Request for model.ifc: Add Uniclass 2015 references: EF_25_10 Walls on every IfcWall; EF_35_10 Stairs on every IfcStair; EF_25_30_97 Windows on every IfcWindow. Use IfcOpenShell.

First a look at what the model holds.

```python
import ifcopenshell

model = ifcopenshell.open("model.ifc")
print(model.schema)
print("classifications:", [c.Name for c in model.by_type("IfcClassification")])
for ifc_class in ("IfcDoor", "IfcRoof", "IfcStair", "IfcWall", "IfcWindow"):
    print(ifc_class, len(model.by_type(ifc_class)))
```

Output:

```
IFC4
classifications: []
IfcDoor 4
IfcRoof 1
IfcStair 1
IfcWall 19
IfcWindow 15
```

```python
import ifcopenshell
import ifcopenshell.api.classification

model = ifcopenshell.open("model.ifc")

system = ifcopenshell.api.classification.add_classification(model, classification="Uniclass 2015")

codes = {
    "IfcWall": ("EF_25_10", "Walls"),
    "IfcStair": ("EF_35_10", "Stairs"),
    "IfcWindow": ("EF_25_30_97", "Windows"),
}
for ifc_class, (code, name) in codes.items():
    products = model.by_type(ifc_class)
    ifcopenshell.api.classification.add_reference(
        model, products=products, classification=system, identification=code, name=name
    )
    print(code, len(products))

model.write("model_rev.ifc")
```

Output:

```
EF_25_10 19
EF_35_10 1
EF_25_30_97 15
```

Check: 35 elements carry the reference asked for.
